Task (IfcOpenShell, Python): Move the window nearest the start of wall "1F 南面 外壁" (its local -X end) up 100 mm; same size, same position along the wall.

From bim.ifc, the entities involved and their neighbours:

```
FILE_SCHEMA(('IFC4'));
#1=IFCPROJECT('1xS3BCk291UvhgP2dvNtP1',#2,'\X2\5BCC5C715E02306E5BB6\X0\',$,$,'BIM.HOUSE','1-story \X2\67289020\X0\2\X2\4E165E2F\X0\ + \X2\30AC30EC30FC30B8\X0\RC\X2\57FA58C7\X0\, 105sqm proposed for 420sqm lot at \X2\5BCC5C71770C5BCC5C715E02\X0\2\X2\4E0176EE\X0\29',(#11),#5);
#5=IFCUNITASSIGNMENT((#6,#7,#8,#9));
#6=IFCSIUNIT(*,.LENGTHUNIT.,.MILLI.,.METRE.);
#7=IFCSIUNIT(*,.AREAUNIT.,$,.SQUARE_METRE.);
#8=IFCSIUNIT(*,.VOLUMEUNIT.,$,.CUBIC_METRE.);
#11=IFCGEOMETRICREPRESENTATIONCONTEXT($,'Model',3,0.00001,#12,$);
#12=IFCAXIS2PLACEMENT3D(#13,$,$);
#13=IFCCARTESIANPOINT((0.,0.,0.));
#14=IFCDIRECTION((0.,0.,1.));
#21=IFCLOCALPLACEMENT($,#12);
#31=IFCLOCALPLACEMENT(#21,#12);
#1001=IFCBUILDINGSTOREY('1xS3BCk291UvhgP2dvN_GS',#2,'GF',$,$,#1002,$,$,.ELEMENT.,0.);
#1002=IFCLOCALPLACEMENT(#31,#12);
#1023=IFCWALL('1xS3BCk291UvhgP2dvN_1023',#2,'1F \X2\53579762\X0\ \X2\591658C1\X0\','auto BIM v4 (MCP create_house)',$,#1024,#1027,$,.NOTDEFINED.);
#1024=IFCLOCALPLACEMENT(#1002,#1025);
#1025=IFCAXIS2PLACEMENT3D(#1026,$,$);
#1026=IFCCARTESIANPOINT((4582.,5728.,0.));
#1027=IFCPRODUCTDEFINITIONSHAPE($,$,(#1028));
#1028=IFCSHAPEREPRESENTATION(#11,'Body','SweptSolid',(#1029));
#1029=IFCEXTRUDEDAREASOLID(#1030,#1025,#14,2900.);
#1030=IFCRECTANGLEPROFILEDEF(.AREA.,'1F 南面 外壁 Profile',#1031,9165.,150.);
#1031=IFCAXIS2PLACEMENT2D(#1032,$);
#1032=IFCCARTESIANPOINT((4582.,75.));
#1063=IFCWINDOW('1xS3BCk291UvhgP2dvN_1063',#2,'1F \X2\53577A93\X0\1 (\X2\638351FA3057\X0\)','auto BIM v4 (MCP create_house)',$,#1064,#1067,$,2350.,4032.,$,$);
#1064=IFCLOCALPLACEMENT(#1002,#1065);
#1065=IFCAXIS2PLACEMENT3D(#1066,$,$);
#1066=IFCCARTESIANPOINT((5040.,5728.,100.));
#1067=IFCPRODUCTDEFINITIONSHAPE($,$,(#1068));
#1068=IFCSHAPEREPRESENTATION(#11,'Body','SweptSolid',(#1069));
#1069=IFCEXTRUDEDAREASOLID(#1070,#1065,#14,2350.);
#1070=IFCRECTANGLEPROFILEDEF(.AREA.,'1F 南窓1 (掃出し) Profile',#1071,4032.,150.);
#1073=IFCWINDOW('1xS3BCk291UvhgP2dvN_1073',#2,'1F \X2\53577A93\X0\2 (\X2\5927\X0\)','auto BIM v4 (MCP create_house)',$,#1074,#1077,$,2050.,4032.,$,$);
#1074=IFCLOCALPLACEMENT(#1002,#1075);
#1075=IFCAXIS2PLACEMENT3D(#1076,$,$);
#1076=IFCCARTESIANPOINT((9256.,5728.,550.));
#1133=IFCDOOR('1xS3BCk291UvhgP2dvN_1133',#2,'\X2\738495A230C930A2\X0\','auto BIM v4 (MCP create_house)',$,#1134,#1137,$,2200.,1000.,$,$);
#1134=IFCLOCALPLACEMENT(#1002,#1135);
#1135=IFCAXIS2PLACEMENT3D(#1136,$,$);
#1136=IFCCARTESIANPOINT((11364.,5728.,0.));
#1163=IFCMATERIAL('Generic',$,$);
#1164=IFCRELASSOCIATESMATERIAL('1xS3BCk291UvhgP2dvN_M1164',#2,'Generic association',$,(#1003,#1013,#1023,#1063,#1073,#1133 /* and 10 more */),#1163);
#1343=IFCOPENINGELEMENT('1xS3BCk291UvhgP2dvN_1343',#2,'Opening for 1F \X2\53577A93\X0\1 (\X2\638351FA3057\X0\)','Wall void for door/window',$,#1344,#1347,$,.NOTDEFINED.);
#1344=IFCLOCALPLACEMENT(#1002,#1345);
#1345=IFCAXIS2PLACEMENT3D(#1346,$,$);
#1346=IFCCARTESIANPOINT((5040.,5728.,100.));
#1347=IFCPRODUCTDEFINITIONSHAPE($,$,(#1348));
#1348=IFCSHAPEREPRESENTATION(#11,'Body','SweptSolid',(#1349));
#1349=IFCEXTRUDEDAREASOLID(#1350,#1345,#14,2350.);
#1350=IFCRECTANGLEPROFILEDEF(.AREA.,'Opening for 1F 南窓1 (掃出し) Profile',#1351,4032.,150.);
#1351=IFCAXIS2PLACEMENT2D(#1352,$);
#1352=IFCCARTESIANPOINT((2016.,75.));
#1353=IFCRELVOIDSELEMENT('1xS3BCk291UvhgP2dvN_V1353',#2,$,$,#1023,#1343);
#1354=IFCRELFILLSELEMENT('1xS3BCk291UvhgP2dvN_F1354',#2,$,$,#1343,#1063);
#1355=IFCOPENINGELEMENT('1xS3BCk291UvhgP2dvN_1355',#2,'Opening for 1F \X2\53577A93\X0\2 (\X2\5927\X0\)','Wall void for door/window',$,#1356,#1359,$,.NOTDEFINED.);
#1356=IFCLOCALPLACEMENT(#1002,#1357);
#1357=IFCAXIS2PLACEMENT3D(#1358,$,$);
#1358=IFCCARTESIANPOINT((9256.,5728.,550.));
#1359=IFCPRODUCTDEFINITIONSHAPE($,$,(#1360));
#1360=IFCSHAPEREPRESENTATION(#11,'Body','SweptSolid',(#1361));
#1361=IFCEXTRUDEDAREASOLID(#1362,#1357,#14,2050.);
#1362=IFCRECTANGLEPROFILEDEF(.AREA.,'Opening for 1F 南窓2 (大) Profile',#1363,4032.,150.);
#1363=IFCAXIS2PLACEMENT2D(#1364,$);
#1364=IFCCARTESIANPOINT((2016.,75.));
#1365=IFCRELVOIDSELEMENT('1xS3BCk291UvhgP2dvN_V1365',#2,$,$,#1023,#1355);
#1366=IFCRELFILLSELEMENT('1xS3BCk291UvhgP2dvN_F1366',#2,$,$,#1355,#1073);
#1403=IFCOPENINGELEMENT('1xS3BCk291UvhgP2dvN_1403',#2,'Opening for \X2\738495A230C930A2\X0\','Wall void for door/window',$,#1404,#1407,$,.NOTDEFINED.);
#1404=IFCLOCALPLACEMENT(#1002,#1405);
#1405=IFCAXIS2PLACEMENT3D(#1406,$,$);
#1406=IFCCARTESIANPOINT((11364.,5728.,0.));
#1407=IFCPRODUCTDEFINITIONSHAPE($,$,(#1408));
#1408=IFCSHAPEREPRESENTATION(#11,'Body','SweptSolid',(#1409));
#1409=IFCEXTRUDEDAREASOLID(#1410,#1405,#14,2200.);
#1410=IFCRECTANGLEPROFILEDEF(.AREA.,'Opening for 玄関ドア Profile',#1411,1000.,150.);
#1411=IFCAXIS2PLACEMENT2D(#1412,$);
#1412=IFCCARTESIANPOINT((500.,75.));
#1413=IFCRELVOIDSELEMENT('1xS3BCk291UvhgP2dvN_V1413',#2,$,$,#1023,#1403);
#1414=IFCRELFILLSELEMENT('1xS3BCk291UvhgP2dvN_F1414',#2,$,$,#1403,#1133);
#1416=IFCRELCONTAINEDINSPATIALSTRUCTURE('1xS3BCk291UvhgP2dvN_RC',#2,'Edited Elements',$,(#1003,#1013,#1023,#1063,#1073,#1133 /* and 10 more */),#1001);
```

```python
import numpy as np
import ifcopenshell
import ifcopenshell.api.geometry
import ifcopenshell.util.placement
import ifcopenshell.util.unit

model = ifcopenshell.open("bim.ifc")
unit_scale = ifcopenshell.util.unit.calculate_unit_scale(model)

window = model.by_guid("1xS3BCk291UvhgP2dvN_1063")
opening = window.FillsVoids[0].RelatingOpeningElement
dz = 0.1 / unit_scale

shift = np.array([0.0, 0.0, dz])
# The window is not placed relative to its opening, so move both.
for product in (opening, window):
    matrix = ifcopenshell.util.placement.get_local_placement(product.ObjectPlacement)
    matrix[:3, 3] += shift
    ifcopenshell.api.geometry.edit_object_placement(model, product=product, matrix=matrix, is_si=False)

print(f"moved by {dz * unit_scale:+.3f} m")

model.write("bim-out.ifc")
```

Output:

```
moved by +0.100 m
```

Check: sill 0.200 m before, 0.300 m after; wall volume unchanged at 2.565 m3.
